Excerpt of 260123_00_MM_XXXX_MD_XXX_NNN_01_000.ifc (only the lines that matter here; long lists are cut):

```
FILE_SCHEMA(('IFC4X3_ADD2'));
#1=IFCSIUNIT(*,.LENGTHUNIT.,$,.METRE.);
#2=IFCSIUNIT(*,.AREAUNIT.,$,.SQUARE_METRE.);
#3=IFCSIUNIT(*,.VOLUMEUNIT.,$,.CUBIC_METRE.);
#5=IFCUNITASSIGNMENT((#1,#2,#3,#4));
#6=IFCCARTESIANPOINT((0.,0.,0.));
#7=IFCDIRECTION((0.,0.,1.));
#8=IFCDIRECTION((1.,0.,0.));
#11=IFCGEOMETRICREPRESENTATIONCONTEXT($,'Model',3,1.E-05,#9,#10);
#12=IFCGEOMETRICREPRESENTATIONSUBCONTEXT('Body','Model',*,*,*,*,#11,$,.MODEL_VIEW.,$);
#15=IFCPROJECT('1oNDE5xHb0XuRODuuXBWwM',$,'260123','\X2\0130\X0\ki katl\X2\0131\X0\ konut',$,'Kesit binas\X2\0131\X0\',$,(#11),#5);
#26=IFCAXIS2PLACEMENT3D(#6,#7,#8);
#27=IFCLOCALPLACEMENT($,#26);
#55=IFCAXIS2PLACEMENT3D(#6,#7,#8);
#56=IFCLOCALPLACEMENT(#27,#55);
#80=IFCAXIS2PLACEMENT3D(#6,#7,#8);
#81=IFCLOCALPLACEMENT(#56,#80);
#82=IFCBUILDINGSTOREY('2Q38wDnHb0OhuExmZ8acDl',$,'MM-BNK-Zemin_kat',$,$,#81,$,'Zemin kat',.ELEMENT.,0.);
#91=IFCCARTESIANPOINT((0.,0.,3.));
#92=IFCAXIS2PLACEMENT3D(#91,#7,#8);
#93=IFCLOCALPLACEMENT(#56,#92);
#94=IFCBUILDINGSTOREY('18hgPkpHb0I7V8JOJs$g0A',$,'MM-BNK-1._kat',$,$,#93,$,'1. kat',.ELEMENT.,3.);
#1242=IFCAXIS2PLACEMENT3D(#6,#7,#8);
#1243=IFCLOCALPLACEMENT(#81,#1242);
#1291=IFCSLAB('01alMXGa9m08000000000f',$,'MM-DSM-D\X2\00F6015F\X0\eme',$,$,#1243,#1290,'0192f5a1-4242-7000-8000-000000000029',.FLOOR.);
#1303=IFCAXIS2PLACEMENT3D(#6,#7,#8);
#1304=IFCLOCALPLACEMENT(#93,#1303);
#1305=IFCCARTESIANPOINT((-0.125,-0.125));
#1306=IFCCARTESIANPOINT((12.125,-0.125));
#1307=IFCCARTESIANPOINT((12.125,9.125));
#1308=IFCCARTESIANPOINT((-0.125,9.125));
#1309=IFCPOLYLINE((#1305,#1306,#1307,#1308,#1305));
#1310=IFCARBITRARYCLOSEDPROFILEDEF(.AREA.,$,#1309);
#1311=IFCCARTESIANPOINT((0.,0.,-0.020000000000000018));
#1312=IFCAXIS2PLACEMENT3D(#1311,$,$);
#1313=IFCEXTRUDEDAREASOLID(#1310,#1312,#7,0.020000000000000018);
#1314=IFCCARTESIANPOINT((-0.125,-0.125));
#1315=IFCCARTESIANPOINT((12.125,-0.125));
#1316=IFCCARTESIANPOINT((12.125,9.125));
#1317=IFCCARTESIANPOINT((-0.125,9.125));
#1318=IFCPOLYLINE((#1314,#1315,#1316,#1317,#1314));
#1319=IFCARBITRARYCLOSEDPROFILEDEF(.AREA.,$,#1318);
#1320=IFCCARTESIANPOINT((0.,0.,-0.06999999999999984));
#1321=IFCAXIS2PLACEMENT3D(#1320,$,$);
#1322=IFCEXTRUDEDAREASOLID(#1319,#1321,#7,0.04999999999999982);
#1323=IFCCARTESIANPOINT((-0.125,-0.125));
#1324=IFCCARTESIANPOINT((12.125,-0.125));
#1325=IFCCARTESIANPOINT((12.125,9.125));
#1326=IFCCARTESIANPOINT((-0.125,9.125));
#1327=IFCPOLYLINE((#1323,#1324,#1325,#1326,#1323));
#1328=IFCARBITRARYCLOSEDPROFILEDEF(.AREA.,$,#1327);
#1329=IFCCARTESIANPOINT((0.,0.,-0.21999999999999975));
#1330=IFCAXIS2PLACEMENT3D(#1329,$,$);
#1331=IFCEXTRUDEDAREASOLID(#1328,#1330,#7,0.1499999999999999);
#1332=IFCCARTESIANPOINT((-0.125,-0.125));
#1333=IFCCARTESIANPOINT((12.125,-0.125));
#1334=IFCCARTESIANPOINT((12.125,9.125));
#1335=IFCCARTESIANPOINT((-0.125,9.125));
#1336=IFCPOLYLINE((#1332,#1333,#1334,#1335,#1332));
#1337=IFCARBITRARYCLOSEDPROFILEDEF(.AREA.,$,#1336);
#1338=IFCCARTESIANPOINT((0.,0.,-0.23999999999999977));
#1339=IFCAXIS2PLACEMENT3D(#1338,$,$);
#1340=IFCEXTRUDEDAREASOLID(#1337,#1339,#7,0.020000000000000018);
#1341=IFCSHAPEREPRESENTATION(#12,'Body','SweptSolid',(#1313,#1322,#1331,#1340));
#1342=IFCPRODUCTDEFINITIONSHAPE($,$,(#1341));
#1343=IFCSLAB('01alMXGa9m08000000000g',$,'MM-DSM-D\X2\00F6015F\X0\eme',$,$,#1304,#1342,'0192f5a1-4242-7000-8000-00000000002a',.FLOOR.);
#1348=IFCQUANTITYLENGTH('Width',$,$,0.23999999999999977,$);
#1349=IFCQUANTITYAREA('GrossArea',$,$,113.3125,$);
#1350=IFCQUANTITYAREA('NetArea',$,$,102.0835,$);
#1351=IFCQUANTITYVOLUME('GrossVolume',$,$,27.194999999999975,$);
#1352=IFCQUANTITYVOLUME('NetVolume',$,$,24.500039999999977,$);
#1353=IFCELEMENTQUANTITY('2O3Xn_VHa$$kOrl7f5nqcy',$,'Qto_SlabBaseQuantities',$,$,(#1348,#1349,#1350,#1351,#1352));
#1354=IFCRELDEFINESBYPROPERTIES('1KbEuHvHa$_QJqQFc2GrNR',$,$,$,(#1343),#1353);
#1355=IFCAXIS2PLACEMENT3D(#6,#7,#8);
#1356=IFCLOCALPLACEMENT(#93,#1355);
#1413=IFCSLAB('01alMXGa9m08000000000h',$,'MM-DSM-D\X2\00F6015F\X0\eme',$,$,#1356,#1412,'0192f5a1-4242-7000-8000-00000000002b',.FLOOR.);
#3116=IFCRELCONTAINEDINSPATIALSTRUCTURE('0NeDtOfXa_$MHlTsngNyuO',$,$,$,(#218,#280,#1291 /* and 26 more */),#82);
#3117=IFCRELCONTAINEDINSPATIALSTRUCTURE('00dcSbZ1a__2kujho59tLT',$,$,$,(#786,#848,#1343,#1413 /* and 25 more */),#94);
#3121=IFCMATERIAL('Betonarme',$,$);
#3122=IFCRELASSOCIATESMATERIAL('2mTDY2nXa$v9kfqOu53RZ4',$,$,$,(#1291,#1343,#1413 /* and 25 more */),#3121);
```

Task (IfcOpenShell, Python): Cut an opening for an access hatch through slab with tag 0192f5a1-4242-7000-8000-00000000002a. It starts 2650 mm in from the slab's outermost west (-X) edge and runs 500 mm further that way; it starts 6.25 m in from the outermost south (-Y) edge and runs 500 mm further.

```python
import numpy as np
import ifcopenshell
import ifcopenshell.api.feature
import ifcopenshell.api.geometry
import ifcopenshell.api.pset
import ifcopenshell.api.root
import ifcopenshell.geom
import ifcopenshell.util.element
import ifcopenshell.util.placement
import ifcopenshell.util.representation
import ifcopenshell.util.shape
import ifcopenshell.util.unit

model = ifcopenshell.open("260123_00_MM_XXXX_MD_XXX_NNN_01_000.ifc")
unit_scale = ifcopenshell.util.unit.calculate_unit_scale(model)
area_scale = ifcopenshell.util.unit.calculate_unit_scale(model, "AREAUNIT")
volume_scale = ifcopenshell.util.unit.calculate_unit_scale(model, "VOLUMEUNIT")
settings = ifcopenshell.geom.settings()


def volume(element):
    """Net volume in cubic metres, openings subtracted."""
    shape = ifcopenshell.geom.create_shape(settings, element)
    return ifcopenshell.util.shape.get_volume(shape.geometry)


slab = model.by_guid("01alMXGa9m08000000000g")
before = volume(slab)

# Extent in the slab's own axes, in metres. The edges named are its -X and -Y sides.
slab_shape = ifcopenshell.geom.create_shape(settings, slab)
vertices = ifcopenshell.util.shape.get_vertices(slab_shape.geometry)
x_min, y_min, bottom = vertices.min(axis=0)
top = vertices[:, 2].max()

opening = ifcopenshell.api.root.create_entity(model, ifc_class="IfcOpeningElement", name="Access hatch opening", predefined_type="OPENING")
context = ifcopenshell.util.representation.get_context(model, "Model", "Body", "MODEL_VIEW")
width, depth = 0.5, 0.5
outline = [(0.0, 0.0), (width, 0.0), (width, depth), (0.0, depth), (0.0, 0.0)]
# Overshoot both faces by 50 mm so the cut is clean.
shape = ifcopenshell.api.geometry.add_slab_representation(
    model, context=context, depth=top - bottom + 0.1, polyline=outline
)
ifcopenshell.api.geometry.assign_representation(model, product=opening, representation=shape)

matrix = ifcopenshell.util.placement.get_local_placement(slab.ObjectPlacement)
matrix[:, 3] = matrix @ np.append(np.array([x_min + 2.65, y_min + 6.25, bottom - 0.05]) / unit_scale, 1.0)
ifcopenshell.api.geometry.edit_object_placement(model, product=opening, matrix=matrix, is_si=False)
ifcopenshell.api.feature.add_feature(model, feature=opening, element=slab)

after = volume(slab)

# Update the slab's stored quantities.
qto = model.by_id(ifcopenshell.util.element.get_pset(slab, "Qto_SlabBaseQuantities", should_inherit=False)["id"])
ifcopenshell.api.pset.edit_qto(model, qto=qto, properties={
    "NetArea": after / (top - bottom) / area_scale,
    "NetVolume": after / volume_scale,
})

print(f"slab volume {before:.3f} -> {after:.3f} m3")

model.write("260123_00_MM_XXXX_MD_XXX_NNN_01_000_edited.ifc")
```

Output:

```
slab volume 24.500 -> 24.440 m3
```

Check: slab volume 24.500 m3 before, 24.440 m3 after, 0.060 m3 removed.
